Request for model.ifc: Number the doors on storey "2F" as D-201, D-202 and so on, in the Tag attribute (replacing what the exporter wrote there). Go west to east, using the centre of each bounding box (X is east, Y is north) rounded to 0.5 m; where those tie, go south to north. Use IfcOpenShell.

First a look at what the model holds.

```python
import ifcopenshell
import ifcopenshell.util.element
import ifcopenshell.util.placement

model = ifcopenshell.open("model.ifc")
print(model.schema)
storey = next(s for s in model.by_type("IfcBuildingStorey") if s.Name == "2F")
doors = [e for e in ifcopenshell.util.element.get_decomposition(storey) if e.is_a("IfcDoor")]
for e in sorted(doors, key=lambda e: e.id()):
    origin = ifcopenshell.util.placement.get_local_placement(e.ObjectPlacement)[:3, 3]
    print(e.id(), e.Tag, e.Name, origin.round(2) + 0.0, sep=" | ")
```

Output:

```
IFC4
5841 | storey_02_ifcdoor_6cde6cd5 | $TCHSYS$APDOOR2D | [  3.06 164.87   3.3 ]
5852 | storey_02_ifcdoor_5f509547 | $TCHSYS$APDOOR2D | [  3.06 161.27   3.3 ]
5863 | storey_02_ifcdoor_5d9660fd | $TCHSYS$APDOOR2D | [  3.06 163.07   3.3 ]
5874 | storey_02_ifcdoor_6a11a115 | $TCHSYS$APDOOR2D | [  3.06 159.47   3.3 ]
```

```python
import ifcopenshell
import ifcopenshell.geom
import ifcopenshell.util.element
import ifcopenshell.util.shape

model = ifcopenshell.open("model.ifc")
settings = ifcopenshell.geom.settings()
settings.set("use-world-coords", True)


def centre(element):
    shape = ifcopenshell.geom.create_shape(settings, element)
    return ifcopenshell.util.shape.get_bbox_centroid(shape.geometry)


storey = next(s for s in model.by_type("IfcBuildingStorey") if s.Name == "2F")
doors = [e for e in ifcopenshell.util.element.get_decomposition(storey) if e.is_a("IfcDoor")]

# Insertion points can sit at a corner or the storey origin, so sort by the geometry (in metres).
centres = {e: centre(e) for e in doors}
doors.sort(key=lambda e: (round(centres[e][0] / 0.5), centres[e][1]))

for i, e in enumerate(doors, start=1):
    number = f"D-2{i:02d}"
    e.Tag = number
    print(e.id(), number)

model.write("model_rev.ifc")
```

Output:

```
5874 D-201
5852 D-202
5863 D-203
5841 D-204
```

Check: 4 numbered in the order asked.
